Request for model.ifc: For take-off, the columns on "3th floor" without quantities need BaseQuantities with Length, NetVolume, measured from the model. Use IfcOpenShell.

First a look at what the model holds.

```python
import ifcopenshell
import ifcopenshell.util.element
import ifcopenshell.util.unit

model = ifcopenshell.open("model.ifc")
print(model.schema)
for unit_type in ("LENGTHUNIT", "AREAUNIT", "VOLUMEUNIT"):
    print(unit_type, ifcopenshell.util.unit.calculate_unit_scale(model, unit_type))
storey = next(s for s in model.by_type("IfcBuildingStorey") if s.Name == "3th floor")
columns = [e for e in ifcopenshell.util.element.get_decomposition(storey) if e.is_a("IfcColumn")]
for e in sorted(columns, key=lambda e: e.id()):
    print(e.id(), e.is_a(), e.Name, list(ifcopenshell.util.element.get_psets(e, qtos_only=True)), sep=" | ")
```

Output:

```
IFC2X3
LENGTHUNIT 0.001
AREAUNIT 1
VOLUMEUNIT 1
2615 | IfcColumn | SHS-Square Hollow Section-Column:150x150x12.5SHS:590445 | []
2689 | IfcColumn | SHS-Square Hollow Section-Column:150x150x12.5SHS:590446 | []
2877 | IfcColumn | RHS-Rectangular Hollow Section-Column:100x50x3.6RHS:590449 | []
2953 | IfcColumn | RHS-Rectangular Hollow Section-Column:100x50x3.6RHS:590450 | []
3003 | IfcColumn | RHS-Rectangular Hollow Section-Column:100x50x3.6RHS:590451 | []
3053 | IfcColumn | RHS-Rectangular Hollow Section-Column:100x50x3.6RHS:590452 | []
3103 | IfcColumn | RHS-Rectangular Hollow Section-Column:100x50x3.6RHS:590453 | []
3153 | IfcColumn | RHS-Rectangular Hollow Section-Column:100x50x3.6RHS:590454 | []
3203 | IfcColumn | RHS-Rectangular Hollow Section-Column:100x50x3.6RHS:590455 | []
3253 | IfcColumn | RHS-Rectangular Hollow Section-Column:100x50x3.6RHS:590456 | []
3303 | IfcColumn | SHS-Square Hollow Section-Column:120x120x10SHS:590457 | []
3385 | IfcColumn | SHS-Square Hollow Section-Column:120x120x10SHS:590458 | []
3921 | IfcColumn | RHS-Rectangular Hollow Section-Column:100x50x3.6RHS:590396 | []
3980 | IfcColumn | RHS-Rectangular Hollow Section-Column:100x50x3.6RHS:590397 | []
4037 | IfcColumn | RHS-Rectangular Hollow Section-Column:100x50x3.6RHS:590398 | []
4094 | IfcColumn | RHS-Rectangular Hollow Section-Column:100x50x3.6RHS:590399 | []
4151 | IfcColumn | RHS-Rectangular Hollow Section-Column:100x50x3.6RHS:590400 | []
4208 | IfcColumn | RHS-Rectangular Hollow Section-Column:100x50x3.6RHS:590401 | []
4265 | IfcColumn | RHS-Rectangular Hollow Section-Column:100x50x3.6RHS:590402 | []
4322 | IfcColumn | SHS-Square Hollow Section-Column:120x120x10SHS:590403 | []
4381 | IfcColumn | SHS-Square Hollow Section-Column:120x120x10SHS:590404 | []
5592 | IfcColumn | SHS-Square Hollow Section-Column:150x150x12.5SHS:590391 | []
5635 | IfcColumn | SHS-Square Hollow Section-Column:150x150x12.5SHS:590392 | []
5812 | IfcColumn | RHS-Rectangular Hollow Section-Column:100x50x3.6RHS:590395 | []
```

```python
import ifcopenshell
import ifcopenshell.api.pset
import ifcopenshell.geom
import ifcopenshell.util.element
import ifcopenshell.util.shape
import ifcopenshell.util.unit

model = ifcopenshell.open("model.ifc")
unit_scale = ifcopenshell.util.unit.calculate_unit_scale(model)
volume_scale = ifcopenshell.util.unit.calculate_unit_scale(model, "VOLUMEUNIT")
settings = ifcopenshell.geom.settings()

storey = next(s for s in model.by_type("IfcBuildingStorey") if s.Name == "3th floor")
columns = [e for e in ifcopenshell.util.element.get_decomposition(storey) if e.is_a("IfcColumn")]

for e in sorted(columns, key=lambda e: e.id()):
    if ifcopenshell.util.element.get_psets(e, qtos_only=True, should_inherit=False):
        continue
    # Geometry comes back in metres, in the element's own axes.
    shape = ifcopenshell.geom.create_shape(settings, e)
    values = {
        "Length": ifcopenshell.util.shape.get_z(shape.geometry) / unit_scale,
        "NetVolume": ifcopenshell.util.shape.get_volume(shape.geometry) / volume_scale,
    }
    qto = ifcopenshell.api.pset.add_qto(model, product=e, name="BaseQuantities")
    ifcopenshell.api.pset.edit_qto(model, qto=qto, properties=values)
    print(e.id(), {k: round(v, 3) for k, v in values.items()})

model.write("model_edited.ifc")
```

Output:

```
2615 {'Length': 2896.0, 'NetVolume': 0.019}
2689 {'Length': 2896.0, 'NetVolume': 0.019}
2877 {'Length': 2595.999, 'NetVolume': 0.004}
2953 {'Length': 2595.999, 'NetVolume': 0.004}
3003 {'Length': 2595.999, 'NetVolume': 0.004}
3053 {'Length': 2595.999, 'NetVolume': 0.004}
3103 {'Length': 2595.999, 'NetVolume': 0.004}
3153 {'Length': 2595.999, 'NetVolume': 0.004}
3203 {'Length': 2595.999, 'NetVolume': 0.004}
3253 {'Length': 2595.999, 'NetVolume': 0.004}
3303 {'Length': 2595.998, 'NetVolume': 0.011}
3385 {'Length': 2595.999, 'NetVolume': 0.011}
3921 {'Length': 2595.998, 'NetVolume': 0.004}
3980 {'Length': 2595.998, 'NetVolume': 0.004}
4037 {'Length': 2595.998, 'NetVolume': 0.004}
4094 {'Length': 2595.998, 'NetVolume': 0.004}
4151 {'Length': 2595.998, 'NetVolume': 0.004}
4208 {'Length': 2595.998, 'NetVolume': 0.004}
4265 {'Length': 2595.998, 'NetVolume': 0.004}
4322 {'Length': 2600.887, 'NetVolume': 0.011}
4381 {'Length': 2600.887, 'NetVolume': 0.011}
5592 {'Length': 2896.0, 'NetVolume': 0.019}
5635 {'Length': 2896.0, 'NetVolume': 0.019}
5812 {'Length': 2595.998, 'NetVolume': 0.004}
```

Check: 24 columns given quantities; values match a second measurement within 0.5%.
